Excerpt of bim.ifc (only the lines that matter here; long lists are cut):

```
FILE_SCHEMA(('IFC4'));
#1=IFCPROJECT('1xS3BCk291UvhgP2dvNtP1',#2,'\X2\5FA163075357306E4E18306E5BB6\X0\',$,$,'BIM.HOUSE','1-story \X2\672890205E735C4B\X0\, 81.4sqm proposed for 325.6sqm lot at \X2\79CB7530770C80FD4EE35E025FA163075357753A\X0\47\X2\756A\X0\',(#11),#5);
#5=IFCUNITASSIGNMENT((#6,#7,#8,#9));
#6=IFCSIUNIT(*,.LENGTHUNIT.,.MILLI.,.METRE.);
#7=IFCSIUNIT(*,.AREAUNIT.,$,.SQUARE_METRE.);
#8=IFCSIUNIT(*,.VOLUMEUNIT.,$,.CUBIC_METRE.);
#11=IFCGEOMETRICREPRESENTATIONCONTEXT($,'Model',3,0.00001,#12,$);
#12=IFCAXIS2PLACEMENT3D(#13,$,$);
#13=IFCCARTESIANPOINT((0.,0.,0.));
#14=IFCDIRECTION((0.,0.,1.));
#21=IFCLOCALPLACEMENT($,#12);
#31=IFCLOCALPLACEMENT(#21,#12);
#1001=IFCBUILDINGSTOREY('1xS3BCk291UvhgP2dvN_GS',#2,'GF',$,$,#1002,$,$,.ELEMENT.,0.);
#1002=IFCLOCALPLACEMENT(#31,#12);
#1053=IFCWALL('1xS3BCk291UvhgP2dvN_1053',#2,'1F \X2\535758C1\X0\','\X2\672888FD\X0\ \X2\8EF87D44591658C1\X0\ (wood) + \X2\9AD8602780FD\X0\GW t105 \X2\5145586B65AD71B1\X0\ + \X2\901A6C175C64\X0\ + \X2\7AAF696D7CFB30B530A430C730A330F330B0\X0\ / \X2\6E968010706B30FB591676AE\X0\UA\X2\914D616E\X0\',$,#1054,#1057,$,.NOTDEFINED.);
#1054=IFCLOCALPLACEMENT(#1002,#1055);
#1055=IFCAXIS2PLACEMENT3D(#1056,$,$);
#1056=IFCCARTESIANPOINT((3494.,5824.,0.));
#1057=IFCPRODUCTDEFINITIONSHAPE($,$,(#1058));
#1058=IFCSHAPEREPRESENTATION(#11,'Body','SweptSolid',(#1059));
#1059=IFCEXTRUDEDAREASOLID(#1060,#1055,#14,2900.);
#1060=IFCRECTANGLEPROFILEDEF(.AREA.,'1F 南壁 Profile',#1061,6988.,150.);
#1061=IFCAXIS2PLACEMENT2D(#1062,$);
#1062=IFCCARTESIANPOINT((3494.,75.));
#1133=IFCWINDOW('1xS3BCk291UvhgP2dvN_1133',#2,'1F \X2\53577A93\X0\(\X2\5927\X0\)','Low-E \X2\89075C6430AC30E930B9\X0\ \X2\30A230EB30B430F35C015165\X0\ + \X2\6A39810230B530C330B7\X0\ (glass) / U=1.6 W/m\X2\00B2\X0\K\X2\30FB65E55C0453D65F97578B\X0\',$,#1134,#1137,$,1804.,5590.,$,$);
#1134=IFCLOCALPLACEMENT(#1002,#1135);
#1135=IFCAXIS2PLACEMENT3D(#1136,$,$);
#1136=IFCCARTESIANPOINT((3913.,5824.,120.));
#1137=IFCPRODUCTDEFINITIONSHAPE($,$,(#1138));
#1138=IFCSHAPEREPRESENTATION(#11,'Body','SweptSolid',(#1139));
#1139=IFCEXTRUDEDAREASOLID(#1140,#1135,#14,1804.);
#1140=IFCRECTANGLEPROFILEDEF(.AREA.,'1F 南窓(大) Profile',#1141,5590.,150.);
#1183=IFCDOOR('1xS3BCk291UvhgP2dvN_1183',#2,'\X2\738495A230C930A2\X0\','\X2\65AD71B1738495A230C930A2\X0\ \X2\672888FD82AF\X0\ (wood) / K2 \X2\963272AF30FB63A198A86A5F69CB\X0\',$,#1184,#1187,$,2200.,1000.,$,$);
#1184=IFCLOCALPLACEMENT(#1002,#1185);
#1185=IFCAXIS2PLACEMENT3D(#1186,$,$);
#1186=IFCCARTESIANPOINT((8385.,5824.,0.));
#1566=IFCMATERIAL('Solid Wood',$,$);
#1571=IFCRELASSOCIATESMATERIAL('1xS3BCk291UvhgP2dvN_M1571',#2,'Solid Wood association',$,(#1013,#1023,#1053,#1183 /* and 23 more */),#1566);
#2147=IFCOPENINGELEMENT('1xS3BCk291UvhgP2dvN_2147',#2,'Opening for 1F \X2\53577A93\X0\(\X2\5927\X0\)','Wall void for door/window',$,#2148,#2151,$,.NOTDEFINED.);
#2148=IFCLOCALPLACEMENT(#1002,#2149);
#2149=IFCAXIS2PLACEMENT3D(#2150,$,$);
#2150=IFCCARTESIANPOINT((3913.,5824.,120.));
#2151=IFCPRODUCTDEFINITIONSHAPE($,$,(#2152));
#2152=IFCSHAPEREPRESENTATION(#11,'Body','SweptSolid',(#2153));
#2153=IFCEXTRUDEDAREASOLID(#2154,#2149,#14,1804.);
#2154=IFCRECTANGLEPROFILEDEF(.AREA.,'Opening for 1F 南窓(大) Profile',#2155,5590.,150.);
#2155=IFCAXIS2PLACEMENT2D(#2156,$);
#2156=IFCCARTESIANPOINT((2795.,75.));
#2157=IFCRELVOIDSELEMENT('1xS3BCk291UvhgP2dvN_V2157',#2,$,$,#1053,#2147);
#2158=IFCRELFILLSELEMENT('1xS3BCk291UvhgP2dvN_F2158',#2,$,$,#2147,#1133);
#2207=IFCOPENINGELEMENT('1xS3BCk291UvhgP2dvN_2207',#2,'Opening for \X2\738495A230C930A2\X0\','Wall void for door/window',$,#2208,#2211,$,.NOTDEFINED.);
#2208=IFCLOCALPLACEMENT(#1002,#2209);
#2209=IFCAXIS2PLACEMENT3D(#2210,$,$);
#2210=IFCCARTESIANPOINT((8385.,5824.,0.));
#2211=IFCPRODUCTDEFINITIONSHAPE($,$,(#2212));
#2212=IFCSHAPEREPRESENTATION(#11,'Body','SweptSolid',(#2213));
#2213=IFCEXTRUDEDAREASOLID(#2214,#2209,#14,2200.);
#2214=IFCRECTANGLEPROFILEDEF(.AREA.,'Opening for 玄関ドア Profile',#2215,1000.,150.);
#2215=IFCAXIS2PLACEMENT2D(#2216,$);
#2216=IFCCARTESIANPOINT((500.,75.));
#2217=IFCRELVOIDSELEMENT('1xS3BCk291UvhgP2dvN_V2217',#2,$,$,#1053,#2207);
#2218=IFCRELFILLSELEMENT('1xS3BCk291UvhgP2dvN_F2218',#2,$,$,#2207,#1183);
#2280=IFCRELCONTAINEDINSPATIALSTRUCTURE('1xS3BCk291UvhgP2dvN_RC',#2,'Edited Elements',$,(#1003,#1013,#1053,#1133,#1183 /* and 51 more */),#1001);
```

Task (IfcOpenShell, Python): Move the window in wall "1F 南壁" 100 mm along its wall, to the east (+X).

```python
import ifcopenshell
import ifcopenshell.api.geometry
import ifcopenshell.util.placement

model = ifcopenshell.open("bim.ifc")

window = model.by_id(1133)
opening = window.FillsVoids[0].RelatingOpeningElement
wall = opening.VoidsElements[0].RelatingBuildingElement

wall_matrix = ifcopenshell.util.placement.get_local_placement(wall.ObjectPlacement)
shift = wall_matrix[:3, 0] * 100.0
before = ifcopenshell.util.placement.get_local_placement(window.ObjectPlacement)[:3, 3].copy()

# The window is not placed relative to its opening, so move both.
for product in (opening, window):
    matrix = ifcopenshell.util.placement.get_local_placement(product.ObjectPlacement)
    matrix[:3, 3] += shift
    ifcopenshell.api.geometry.edit_object_placement(model, product=product, matrix=matrix, is_si=False)

after = ifcopenshell.util.placement.get_local_placement(window.ObjectPlacement)[:3, 3]
print("window moved by", (after - before).round(3) + 0.0)

model.write("bim_updated.ifc")
```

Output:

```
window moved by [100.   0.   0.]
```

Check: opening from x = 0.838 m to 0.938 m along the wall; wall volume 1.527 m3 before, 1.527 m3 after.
